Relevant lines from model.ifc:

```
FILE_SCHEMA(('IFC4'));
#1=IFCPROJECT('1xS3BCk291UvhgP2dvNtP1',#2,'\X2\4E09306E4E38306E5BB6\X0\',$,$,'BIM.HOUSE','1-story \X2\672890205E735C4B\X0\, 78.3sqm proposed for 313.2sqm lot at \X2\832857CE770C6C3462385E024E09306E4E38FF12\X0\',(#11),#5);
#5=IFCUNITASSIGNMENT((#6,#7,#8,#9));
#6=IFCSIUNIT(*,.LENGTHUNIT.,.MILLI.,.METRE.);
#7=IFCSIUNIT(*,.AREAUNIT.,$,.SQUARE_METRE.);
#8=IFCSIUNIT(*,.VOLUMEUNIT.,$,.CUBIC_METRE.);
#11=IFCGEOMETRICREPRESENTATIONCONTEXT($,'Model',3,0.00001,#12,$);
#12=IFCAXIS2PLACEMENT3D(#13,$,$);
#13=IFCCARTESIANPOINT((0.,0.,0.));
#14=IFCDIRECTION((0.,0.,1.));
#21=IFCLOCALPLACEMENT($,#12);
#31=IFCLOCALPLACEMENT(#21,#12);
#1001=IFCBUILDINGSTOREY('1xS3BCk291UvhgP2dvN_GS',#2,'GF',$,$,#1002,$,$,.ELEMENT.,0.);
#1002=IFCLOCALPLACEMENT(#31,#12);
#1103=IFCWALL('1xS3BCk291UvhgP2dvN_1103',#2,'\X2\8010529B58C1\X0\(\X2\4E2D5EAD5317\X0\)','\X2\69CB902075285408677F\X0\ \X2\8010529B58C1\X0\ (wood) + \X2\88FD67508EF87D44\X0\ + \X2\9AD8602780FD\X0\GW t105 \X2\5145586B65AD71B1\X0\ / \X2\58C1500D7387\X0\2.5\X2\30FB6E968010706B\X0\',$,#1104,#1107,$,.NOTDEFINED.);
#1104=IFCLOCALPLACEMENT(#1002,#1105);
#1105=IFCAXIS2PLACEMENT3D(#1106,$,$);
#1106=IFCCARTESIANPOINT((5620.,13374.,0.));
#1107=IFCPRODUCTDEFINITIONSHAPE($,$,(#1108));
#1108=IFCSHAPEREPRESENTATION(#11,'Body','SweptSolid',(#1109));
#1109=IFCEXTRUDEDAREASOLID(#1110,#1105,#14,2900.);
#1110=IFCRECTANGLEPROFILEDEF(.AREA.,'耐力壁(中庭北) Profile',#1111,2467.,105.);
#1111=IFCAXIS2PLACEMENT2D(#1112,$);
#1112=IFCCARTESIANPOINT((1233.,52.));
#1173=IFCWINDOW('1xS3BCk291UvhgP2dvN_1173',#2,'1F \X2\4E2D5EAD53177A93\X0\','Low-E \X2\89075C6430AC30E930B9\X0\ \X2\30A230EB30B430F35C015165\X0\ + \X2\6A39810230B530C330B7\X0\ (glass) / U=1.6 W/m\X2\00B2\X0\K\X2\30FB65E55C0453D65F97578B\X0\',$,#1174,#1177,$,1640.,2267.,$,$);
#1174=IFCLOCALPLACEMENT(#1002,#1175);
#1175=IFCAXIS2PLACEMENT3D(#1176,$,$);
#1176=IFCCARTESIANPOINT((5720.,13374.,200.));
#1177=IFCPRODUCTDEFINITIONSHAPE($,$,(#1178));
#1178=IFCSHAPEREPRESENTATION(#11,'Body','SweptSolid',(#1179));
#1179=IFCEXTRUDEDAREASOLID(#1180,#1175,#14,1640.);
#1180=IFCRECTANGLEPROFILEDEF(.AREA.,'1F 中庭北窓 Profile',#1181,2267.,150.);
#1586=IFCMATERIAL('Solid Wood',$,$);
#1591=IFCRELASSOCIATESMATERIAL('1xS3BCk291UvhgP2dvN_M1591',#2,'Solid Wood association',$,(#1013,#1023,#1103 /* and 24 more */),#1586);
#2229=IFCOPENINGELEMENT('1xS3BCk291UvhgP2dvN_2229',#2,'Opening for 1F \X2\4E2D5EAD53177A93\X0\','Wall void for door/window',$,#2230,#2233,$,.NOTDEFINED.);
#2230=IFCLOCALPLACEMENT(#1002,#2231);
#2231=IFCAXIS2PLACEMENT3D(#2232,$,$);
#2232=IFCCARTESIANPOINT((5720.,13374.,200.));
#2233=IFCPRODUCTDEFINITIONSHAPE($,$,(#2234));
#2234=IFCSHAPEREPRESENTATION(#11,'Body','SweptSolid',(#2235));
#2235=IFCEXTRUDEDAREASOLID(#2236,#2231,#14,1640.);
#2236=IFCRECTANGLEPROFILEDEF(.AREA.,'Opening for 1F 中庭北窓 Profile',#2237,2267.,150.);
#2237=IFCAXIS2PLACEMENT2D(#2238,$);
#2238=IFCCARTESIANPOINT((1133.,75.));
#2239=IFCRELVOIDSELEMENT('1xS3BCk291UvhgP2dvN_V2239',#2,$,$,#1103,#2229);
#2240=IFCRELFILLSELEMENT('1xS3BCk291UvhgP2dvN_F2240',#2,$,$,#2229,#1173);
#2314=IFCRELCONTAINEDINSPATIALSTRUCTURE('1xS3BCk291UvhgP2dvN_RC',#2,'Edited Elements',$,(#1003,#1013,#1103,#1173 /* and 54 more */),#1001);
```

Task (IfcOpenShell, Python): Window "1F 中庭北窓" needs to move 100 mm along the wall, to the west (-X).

```python
import ifcopenshell
import ifcopenshell.api.geometry
import ifcopenshell.util.placement

model = ifcopenshell.open("model.ifc")

window = model.by_guid("1xS3BCk291UvhgP2dvN_1173")
opening = window.FillsVoids[0].RelatingOpeningElement
wall = opening.VoidsElements[0].RelatingBuildingElement

wall_matrix = ifcopenshell.util.placement.get_local_placement(wall.ObjectPlacement)
shift = wall_matrix[:3, 0] * -100.0
before = ifcopenshell.util.placement.get_local_placement(window.ObjectPlacement)[:3, 3].copy()

# The window is not placed relative to its opening, so move both.
for product in (opening, window):
    matrix = ifcopenshell.util.placement.get_local_placement(product.ObjectPlacement)
    matrix[:3, 3] += shift
    ifcopenshell.api.geometry.edit_object_placement(model, product=product, matrix=matrix, is_si=False)

after = ifcopenshell.util.placement.get_local_placement(window.ObjectPlacement)[:3, 3]
print("window moved by", (after - before).round(3) + 0.0)

model.write("model_rev.ifc")
```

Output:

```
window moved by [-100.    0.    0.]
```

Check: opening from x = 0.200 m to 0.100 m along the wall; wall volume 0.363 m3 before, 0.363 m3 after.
